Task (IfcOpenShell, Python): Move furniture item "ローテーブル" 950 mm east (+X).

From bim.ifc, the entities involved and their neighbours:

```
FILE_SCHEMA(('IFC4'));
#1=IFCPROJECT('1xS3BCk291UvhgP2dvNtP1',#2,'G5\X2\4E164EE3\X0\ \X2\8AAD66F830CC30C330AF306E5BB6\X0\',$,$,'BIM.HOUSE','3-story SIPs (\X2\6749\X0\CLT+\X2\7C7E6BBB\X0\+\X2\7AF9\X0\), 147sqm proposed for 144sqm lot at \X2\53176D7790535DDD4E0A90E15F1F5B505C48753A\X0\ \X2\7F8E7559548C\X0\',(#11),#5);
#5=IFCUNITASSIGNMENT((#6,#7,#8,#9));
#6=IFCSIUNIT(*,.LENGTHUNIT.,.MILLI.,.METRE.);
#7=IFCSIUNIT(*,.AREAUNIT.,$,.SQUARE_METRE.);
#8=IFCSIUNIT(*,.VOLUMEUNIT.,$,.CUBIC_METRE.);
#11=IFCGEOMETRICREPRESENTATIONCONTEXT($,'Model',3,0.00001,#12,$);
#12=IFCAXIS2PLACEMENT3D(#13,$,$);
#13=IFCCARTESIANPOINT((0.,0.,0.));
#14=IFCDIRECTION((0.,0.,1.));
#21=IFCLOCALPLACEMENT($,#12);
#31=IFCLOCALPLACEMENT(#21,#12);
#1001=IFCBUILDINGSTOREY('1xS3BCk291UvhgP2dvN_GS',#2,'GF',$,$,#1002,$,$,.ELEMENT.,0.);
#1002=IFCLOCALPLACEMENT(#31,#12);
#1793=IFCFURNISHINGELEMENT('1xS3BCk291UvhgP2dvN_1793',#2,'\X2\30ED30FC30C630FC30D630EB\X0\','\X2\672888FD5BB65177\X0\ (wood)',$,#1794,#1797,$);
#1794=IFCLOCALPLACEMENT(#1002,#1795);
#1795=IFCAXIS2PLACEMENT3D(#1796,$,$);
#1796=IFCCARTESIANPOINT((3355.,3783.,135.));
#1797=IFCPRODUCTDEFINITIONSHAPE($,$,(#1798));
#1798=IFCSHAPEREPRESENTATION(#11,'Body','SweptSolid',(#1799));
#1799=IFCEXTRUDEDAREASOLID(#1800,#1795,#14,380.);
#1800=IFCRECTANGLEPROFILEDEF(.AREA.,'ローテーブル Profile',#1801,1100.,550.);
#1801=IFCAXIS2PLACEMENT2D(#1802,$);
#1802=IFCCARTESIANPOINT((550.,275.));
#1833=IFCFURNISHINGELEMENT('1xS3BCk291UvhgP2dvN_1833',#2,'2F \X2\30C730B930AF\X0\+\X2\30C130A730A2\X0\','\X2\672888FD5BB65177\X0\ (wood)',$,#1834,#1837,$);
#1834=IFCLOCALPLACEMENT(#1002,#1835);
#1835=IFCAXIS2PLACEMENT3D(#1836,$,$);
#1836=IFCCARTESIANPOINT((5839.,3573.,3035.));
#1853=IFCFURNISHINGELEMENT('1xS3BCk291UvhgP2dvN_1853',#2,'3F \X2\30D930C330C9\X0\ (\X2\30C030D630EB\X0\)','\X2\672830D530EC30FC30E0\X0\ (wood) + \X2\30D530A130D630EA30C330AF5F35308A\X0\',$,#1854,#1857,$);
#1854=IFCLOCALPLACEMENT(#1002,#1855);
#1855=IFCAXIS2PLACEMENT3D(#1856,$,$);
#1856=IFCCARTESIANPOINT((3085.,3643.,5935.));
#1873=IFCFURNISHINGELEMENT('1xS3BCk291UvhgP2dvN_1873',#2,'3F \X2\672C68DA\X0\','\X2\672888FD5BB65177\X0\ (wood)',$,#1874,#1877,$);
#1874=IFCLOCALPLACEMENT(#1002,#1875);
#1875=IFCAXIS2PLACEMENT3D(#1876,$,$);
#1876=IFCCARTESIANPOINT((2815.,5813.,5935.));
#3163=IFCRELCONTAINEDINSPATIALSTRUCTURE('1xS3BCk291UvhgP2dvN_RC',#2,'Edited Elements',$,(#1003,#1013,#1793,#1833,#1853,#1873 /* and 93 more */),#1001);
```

```python
import ifcopenshell
import ifcopenshell.api.geometry
import ifcopenshell.util.placement

model = ifcopenshell.open("bim.ifc")

item = model.by_guid("1xS3BCk291UvhgP2dvN_1793")
matrix = ifcopenshell.util.placement.get_local_placement(item.ObjectPlacement)
matrix[0, 3] += 950.0
ifcopenshell.api.geometry.edit_object_placement(model, product=item, matrix=matrix, is_si=False)

print(ifcopenshell.util.placement.get_local_placement(item.ObjectPlacement).round(3) + 0.0)

model.write("bim_v2.ifc")
```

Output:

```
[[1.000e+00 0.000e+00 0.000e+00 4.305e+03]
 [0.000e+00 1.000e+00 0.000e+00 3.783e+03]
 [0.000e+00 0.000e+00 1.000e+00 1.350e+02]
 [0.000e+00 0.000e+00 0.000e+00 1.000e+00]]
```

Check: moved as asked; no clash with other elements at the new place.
